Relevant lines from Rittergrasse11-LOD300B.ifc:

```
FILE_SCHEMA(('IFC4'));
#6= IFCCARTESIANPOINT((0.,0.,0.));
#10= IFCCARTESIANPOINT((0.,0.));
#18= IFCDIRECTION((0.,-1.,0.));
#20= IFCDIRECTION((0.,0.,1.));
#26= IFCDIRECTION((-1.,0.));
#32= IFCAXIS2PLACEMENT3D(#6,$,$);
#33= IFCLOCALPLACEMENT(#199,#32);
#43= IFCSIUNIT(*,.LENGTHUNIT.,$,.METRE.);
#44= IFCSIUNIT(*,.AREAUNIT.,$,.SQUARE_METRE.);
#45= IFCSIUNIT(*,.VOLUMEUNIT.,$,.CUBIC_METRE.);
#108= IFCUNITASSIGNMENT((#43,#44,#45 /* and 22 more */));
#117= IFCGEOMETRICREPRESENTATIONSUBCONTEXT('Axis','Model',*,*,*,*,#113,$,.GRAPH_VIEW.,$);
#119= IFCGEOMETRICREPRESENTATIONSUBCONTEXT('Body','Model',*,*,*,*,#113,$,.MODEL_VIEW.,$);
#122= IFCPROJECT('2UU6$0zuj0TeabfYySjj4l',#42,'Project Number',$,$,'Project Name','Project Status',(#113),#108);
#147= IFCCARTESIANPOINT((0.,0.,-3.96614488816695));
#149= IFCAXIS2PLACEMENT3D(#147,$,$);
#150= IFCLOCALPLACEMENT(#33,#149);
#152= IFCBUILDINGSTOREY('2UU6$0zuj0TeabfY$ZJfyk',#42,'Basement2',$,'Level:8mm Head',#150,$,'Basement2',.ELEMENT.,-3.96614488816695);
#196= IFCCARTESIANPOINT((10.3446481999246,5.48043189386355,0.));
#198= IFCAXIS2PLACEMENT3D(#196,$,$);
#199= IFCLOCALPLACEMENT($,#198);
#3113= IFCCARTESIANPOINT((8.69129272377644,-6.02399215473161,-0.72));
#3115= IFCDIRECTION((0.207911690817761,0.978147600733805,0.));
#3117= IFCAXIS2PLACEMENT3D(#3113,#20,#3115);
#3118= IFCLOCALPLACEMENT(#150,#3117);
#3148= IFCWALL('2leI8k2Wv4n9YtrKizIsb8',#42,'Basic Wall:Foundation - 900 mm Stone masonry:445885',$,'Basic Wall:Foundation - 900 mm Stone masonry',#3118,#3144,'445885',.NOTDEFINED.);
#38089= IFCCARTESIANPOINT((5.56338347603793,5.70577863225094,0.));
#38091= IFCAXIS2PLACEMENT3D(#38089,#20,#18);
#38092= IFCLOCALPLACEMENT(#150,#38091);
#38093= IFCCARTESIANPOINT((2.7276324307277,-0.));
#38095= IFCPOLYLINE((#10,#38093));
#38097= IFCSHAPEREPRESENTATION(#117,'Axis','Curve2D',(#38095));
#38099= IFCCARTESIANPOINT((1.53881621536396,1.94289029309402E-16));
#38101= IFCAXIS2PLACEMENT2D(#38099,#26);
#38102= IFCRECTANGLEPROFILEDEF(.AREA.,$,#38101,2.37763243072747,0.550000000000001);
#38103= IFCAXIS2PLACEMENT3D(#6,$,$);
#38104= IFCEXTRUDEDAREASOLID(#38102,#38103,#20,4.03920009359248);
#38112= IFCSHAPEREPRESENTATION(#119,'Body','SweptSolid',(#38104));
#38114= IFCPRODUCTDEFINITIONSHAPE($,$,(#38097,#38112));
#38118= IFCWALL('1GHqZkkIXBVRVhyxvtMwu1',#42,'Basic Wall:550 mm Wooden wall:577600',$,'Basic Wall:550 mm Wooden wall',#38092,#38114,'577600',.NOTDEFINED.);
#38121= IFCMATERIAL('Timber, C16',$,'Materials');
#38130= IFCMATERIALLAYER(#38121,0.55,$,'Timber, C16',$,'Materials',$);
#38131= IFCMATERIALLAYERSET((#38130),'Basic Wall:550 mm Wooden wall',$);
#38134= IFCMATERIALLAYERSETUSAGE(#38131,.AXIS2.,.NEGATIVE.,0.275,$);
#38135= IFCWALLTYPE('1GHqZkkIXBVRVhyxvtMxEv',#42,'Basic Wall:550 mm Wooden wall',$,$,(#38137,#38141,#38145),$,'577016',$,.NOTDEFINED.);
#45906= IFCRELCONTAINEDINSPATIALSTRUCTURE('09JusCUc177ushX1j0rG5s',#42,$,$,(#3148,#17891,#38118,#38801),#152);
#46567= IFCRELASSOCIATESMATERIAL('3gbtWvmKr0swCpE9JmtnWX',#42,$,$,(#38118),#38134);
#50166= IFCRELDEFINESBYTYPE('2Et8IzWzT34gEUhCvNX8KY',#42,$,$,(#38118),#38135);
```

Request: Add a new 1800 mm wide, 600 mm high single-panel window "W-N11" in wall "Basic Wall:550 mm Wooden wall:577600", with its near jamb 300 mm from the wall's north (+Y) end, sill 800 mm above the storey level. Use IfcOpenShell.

```python
import numpy as np
import ifcopenshell
import ifcopenshell.api.feature
import ifcopenshell.api.geometry
import ifcopenshell.api.root
import ifcopenshell.api.spatial
import ifcopenshell.geom
import ifcopenshell.util.element
import ifcopenshell.util.placement
import ifcopenshell.util.representation
import ifcopenshell.util.shape
import ifcopenshell.util.unit

model = ifcopenshell.open("Rittergrasse11-LOD300B.ifc")
unit_scale = ifcopenshell.util.unit.calculate_unit_scale(model)
settings = ifcopenshell.geom.settings()


def volume(element):
    """Net volume in cubic metres, openings subtracted."""
    shape = ifcopenshell.geom.create_shape(settings, element)
    return ifcopenshell.util.shape.get_volume(shape.geometry)


wall = model.by_guid("1GHqZkkIXBVRVhyxvtMwu1")
storey = ifcopenshell.util.element.get_container(wall, ifc_class="IfcBuildingStorey")
context = ifcopenshell.util.representation.get_context(model, "Model", "Body", "MODEL_VIEW")
before = volume(wall)

width, height, from_end, sill = 1.8, 0.6, 0.3, 0.8  # metres

# The wall runs along its own X axis, and the end named is its -X end.
wall_shape = ifcopenshell.geom.create_shape(settings, wall)
x, y, z = ifcopenshell.util.shape.get_vertices(wall_shape.geometry).T
start = x.min() + from_end
face, thickness = float(y.min()), float(y.max() - y.min())
wall_matrix = ifcopenshell.util.placement.get_local_placement(wall.ObjectPlacement)
level = ifcopenshell.util.placement.get_local_placement(storey.ObjectPlacement)[2, 3]


def in_wall(x, y):
    """Placement at x, y metres in the wall's axes, at sill height."""
    matrix = wall_matrix.copy()
    matrix[:, 3] = wall_matrix @ np.array([x / unit_scale, y / unit_scale, 0.0, 1.0])
    matrix[2, 3] = level + sill / unit_scale
    return matrix


# Opening: a box that overshoots both wall faces by 50 mm.
opening = ifcopenshell.api.root.create_entity(model, ifc_class="IfcOpeningElement", predefined_type="OPENING")
box = ifcopenshell.api.geometry.add_wall_representation(
    model, context=context, length=width, height=height, thickness=thickness + 0.1
)
ifcopenshell.api.geometry.assign_representation(model, product=opening, representation=box)
ifcopenshell.api.geometry.edit_object_placement(model, product=opening, matrix=in_wall(start, face - 0.05), is_si=False)
ifcopenshell.api.feature.add_feature(model, feature=opening, element=wall)

window = ifcopenshell.api.root.create_entity(model, ifc_class="IfcWindow", name="W-N11", predefined_type="WINDOW")
window.OverallWidth, window.OverallHeight = width / unit_scale, height / unit_scale
window.PartitioningType = "SINGLE_PANEL"
body = ifcopenshell.api.geometry.add_window_representation(
    model,
    context=context,
    overall_width=window.OverallWidth,
    overall_height=window.OverallHeight,
    partition_type="SINGLE_PANEL",
)
ifcopenshell.api.geometry.assign_representation(model, product=window, representation=body)
ifcopenshell.api.spatial.assign_container(model, products=[window], relating_structure=storey)
ifcopenshell.api.feature.add_filling(model, opening=opening, element=window)

# Centre the window in the wall's thickness.
ifcopenshell.api.geometry.edit_object_placement(model, product=window, matrix=in_wall(start, face), is_si=False)
window_shape = ifcopenshell.geom.create_shape(settings, window)
depth = ifcopenshell.util.shape.get_vertices(window_shape.geometry)[:, 1]
offset = face + thickness / 2 - (depth.min() + depth.max()) / 2
ifcopenshell.api.geometry.edit_object_placement(model, product=window, matrix=in_wall(start, offset), is_si=False)

after = volume(wall)

print(f"wall volume {before:.3f} -> {after:.3f} m3")

model.write("Rittergrasse11-LOD300B-out.ifc")
```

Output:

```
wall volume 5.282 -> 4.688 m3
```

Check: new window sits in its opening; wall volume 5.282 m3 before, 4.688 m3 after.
